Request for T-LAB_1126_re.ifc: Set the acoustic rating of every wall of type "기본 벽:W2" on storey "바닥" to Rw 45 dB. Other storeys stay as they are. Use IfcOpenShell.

First a look at what the model holds.

```python
import ifcopenshell
import ifcopenshell.util.element

model = ifcopenshell.open("T-LAB_1126_re.ifc")
print(model.schema)
storey = next(s for s in model.by_type("IfcBuildingStorey") if s.Name == "바닥")
walls = [e for e in ifcopenshell.util.element.get_decomposition(storey) if e.is_a("IfcWall")]
seen = {}
for e in walls:
    element_type = ifcopenshell.util.element.get_type(e)
    key = (element_type.Name if element_type != e and element_type else None, ifcopenshell.util.element.get_pset(e, "Pset_WallCommon", "AcousticRating"))
    seen[key] = seen.get(key, 0) + 1
for (name, value), count in sorted(seen.items(), key=str):
    print(count, "x", name, "|", value)
```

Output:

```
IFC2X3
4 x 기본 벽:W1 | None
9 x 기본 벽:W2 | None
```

```python
import ifcopenshell
import ifcopenshell.api.pset
import ifcopenshell.util.element

model = ifcopenshell.open("T-LAB_1126_re.ifc")

storey = next(s for s in model.by_type("IfcBuildingStorey") if s.Name == "바닥")
walls = [e for e in ifcopenshell.util.element.get_decomposition(storey) if e.is_a("IfcWall")]

count = 0
for e in walls:
    element_type = ifcopenshell.util.element.get_type(e)
    if element_type in (None, e) or element_type.Name != "기본 벽:W2":
        continue
    # add_pset returns the element's existing set when there is one.
    pset = ifcopenshell.api.pset.add_pset(model, product=e, name="Pset_WallCommon")
    ifcopenshell.api.pset.edit_pset(model, pset=pset, properties={"AcousticRating": "Rw 45 dB"})
    count += 1

print(count, "walls updated")

model.write("T-LAB_1126_re_edited.ifc")
```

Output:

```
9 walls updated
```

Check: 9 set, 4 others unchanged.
